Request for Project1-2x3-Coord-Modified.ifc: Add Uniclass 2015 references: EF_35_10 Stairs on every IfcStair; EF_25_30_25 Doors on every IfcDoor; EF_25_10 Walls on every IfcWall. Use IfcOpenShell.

First a look at what the model holds.

```python
import ifcopenshell

model = ifcopenshell.open("Project1-2x3-Coord-Modified.ifc")
print(model.schema)
print("classifications:", [c.Name for c in model.by_type("IfcClassification")])
for ifc_class in ("IfcDoor", "IfcRoof", "IfcStair", "IfcWall", "IfcWindow"):
    print(ifc_class, len(model.by_type(ifc_class)))
```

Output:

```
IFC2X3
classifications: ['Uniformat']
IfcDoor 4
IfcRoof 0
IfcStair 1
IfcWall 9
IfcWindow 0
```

```python
import ifcopenshell
import ifcopenshell.api.classification

model = ifcopenshell.open("Project1-2x3-Coord-Modified.ifc")

# IFC2X3 requires Source and Edition and has no link from the project to the system.
system = model.create_entity("IfcClassification", Source="NBS", Edition="2015", Name="Uniclass 2015")

codes = {
    "IfcStair": ("EF_35_10", "Stairs"),
    "IfcDoor": ("EF_25_30_25", "Doors"),
    "IfcWall": ("EF_25_10", "Walls"),
}
for ifc_class, (code, name) in codes.items():
    products = model.by_type(ifc_class)
    ifcopenshell.api.classification.add_reference(
        model, products=products, classification=system, identification=code, name=name
    )
    print(code, len(products))

model.write("Project1-2x3-Coord-Modified_edited.ifc")
```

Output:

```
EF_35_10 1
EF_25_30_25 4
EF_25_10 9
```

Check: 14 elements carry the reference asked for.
